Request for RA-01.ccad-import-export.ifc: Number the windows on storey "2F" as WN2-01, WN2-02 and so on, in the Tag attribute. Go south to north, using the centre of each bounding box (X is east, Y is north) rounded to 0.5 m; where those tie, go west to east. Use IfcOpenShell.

First a look at what the model holds.

```python
import ifcopenshell
import ifcopenshell.util.element
import ifcopenshell.util.placement

model = ifcopenshell.open("RA-01.ccad-import-export.ifc")
print(model.schema)
storey = next(s for s in model.by_type("IfcBuildingStorey") if s.Name == "2F")
windows = [e for e in ifcopenshell.util.element.get_decomposition(storey) if e.is_a("IfcWindow")]
for e in sorted(windows, key=lambda e: e.id()):
    origin = ifcopenshell.util.placement.get_local_placement(e.ObjectPlacement)[:3, 3]
    print(e.id(), e.Tag, e.Name, origin.round(2) + 0.0, sep=" | ")
```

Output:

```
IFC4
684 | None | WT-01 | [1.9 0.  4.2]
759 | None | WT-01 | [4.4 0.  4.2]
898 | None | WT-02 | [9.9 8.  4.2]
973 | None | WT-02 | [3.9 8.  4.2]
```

```python
import ifcopenshell
import ifcopenshell.geom
import ifcopenshell.util.element
import ifcopenshell.util.shape

model = ifcopenshell.open("RA-01.ccad-import-export.ifc")
settings = ifcopenshell.geom.settings()
settings.set("use-world-coords", True)


def centre(element):
    shape = ifcopenshell.geom.create_shape(settings, element)
    return ifcopenshell.util.shape.get_bbox_centroid(shape.geometry)


storey = next(s for s in model.by_type("IfcBuildingStorey") if s.Name == "2F")
windows = [e for e in ifcopenshell.util.element.get_decomposition(storey) if e.is_a("IfcWindow")]

# Insertion points can sit at a corner or the storey origin, so sort by the geometry (in metres).
centres = {e: centre(e) for e in windows}
windows.sort(key=lambda e: (round(centres[e][1] / 0.5), centres[e][0]))

for i, e in enumerate(windows, start=1):
    number = f"WN2-{i:02d}"
    e.Tag = number
    print(e.id(), number)

model.write("RA-01.ccad-import-export_updated.ifc")
```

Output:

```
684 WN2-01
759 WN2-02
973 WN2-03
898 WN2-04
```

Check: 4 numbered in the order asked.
